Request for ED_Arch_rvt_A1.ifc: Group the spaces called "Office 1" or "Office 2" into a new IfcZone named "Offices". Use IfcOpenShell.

First a look at what the model holds.

```python
import ifcopenshell

model = ifcopenshell.open("ED_Arch_rvt_A1.ifc")
print(model.schema)
seen = {}
for space in model.by_type("IfcSpace"):
    seen[space.LongName] = seen.get(space.LongName, 0) + 1
for name, count in sorted(seen.items(), key=str):
    print(count, "x", name)
print("zones:", [z.Name for z in model.by_type("IfcZone")][:20])
```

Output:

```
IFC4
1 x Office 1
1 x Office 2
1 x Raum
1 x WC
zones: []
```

```python
import ifcopenshell
import ifcopenshell.api.group
import ifcopenshell.api.root

model = ifcopenshell.open("ED_Arch_rvt_A1.ifc")

names = {"Office 1", "Office 2"}
spaces = [s for s in model.by_type("IfcSpace") if s.LongName in names]

zone = ifcopenshell.api.root.create_entity(model, ifc_class="IfcZone", name="Offices")
ifcopenshell.api.group.assign_group(model, products=spaces, group=zone)
print(len(spaces), "spaces in", zone.Name)

model.write("ED_Arch_rvt_A1-out.ifc")
```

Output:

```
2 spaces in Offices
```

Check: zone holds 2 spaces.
